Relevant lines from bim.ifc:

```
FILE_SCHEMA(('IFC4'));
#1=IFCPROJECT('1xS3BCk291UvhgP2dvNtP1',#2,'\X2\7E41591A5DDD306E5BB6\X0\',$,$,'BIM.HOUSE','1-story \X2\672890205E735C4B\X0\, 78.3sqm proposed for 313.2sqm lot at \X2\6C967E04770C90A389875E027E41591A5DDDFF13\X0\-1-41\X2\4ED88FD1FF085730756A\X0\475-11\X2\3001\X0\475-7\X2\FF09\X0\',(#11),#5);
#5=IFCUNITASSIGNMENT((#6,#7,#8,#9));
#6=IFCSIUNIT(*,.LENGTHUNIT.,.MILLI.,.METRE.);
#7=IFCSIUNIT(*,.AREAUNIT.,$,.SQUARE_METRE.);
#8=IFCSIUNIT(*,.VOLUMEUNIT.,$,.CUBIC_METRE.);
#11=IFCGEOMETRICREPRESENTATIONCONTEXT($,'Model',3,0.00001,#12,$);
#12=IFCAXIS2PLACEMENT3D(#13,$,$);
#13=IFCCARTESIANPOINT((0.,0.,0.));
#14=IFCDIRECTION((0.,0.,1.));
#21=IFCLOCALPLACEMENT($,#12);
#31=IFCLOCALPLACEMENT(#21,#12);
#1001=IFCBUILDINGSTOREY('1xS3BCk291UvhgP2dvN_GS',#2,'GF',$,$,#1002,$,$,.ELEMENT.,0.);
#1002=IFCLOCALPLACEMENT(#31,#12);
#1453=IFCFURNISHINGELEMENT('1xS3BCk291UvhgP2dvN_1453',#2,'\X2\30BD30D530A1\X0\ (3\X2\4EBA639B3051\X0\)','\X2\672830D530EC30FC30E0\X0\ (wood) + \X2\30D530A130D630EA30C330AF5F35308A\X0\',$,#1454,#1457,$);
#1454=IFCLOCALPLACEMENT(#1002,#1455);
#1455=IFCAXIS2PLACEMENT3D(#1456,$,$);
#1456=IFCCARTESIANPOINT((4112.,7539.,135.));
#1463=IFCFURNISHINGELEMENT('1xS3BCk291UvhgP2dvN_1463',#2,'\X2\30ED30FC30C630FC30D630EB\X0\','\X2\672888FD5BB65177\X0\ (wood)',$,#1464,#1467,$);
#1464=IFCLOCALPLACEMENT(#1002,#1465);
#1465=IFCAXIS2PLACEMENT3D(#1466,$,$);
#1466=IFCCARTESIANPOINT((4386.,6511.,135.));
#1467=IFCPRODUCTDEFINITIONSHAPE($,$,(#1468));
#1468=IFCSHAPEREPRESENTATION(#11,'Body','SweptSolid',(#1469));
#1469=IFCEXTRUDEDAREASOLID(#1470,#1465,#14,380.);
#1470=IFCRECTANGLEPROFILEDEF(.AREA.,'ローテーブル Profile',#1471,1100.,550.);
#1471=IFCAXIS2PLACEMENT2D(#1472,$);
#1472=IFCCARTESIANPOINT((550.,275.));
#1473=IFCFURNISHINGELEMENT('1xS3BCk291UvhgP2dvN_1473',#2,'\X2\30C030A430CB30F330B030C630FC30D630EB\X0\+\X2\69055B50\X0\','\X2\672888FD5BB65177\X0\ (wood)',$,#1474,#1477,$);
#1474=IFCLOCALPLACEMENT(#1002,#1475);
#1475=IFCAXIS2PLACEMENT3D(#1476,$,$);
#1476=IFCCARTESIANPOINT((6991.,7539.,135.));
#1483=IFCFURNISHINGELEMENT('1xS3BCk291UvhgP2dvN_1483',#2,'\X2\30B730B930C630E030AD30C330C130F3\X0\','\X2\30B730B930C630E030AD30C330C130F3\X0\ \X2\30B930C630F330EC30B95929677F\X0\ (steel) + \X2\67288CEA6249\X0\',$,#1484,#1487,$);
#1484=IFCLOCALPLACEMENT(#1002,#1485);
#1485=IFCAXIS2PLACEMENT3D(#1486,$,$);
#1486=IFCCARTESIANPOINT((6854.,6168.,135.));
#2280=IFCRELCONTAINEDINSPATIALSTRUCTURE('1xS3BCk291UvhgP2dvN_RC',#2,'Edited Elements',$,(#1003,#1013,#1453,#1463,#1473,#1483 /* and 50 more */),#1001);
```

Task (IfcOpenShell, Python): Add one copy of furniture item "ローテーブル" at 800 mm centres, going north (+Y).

```python
import numpy as np
import ifcopenshell
import ifcopenshell.api.geometry
import ifcopenshell.api.root
import ifcopenshell.util.element
import ifcopenshell.util.placement
import ifcopenshell.util.unit

model = ifcopenshell.open("bim.ifc")
unit_scale = ifcopenshell.util.unit.calculate_unit_scale(model)


def reuse_history(source, copy):
    """copy_class also copies each property set's owner history, people and application; keep the originals."""
    for rel in copy.IsDefinedBy:
        if rel.is_a("IfcRelDefinesByProperties") and (history := rel.RelatingPropertyDefinition.OwnerHistory):
            rel.RelatingPropertyDefinition.OwnerHistory = source.OwnerHistory
            ifcopenshell.util.element.remove_deep2(model, history)


source = model.by_guid("1xS3BCk291UvhgP2dvN_1463")
base = ifcopenshell.util.placement.get_local_placement(source.ObjectPlacement)
step = np.array([0.0, 1.0, 0.0]) * 0.8 / unit_scale

for i in range(1, 2):
    copy = ifcopenshell.api.root.copy_class(model, product=source)
    copy.Representation = ifcopenshell.util.element.copy_deep(
        model, source.Representation, exclude=["IfcGeometricRepresentationContext", "IfcRepresentationMap"]
    )
    reuse_history(source, copy)
    matrix = base.copy()
    matrix[:3, 3] += i * step
    print("added at", matrix[:3, 3].round(3) + 0.0)
    ifcopenshell.api.geometry.edit_object_placement(model, product=copy, matrix=matrix, is_si=False)

model.write("bim_updated.ifc")
```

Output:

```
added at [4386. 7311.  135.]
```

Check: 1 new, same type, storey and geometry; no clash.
